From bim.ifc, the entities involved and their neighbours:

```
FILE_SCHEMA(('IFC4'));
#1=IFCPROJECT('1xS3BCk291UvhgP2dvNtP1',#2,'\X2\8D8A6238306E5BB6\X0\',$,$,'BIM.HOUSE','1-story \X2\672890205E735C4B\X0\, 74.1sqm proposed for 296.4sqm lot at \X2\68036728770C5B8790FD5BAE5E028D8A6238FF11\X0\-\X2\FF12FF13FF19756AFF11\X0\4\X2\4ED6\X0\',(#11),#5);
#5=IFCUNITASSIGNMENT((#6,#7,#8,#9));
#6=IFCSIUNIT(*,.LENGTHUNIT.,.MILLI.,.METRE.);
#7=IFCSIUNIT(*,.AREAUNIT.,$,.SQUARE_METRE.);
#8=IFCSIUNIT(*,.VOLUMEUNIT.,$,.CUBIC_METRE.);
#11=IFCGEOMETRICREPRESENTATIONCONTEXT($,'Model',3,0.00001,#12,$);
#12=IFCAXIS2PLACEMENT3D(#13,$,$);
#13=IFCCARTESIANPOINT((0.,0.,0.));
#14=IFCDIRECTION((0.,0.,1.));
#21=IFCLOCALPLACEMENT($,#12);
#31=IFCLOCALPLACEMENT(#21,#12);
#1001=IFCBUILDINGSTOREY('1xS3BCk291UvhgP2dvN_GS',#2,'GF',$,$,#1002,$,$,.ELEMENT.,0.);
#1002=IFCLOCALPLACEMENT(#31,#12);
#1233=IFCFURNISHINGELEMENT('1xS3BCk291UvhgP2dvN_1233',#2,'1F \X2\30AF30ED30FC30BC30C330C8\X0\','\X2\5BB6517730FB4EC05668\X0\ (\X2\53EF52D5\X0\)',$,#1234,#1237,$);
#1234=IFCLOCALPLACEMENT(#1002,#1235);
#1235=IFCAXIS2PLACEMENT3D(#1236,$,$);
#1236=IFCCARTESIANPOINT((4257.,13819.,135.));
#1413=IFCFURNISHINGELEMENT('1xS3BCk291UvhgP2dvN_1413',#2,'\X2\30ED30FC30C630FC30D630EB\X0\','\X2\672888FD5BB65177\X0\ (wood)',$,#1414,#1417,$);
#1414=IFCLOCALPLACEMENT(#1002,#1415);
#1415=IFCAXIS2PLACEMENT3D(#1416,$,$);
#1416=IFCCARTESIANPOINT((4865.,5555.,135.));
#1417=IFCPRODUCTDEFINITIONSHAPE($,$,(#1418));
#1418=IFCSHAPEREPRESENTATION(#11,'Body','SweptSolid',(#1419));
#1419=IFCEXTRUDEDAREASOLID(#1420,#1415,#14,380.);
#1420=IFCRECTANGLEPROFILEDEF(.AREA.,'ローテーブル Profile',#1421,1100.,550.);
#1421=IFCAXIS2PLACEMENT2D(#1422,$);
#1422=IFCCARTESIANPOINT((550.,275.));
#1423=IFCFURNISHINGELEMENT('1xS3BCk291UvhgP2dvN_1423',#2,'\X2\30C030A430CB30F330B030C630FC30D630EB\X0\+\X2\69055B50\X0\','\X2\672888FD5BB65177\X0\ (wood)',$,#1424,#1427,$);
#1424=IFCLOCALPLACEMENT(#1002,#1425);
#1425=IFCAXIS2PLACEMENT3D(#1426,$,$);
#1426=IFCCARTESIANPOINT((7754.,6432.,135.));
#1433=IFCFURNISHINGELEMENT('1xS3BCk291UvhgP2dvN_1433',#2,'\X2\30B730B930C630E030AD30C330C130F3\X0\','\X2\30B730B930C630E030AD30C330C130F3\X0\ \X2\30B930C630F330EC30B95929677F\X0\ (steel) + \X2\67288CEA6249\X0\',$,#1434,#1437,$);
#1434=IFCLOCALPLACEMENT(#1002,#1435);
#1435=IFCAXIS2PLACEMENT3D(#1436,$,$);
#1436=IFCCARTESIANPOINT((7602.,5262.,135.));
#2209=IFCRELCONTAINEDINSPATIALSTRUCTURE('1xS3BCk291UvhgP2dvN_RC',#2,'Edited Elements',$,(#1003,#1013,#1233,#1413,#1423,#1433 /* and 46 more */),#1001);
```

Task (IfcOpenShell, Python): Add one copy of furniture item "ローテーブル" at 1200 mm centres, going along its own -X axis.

```python
import ifcopenshell
import ifcopenshell.api.geometry
import ifcopenshell.api.root
import ifcopenshell.util.element
import ifcopenshell.util.placement

model = ifcopenshell.open("bim.ifc")


def reuse_history(source, copy):
    """copy_class also copies each property set's owner history, people and application; keep the originals."""
    for rel in copy.IsDefinedBy:
        if rel.is_a("IfcRelDefinesByProperties") and (history := rel.RelatingPropertyDefinition.OwnerHistory):
            rel.RelatingPropertyDefinition.OwnerHistory = source.OwnerHistory
            ifcopenshell.util.element.remove_deep2(model, history)


source = model.by_guid("1xS3BCk291UvhgP2dvN_1413")
base = ifcopenshell.util.placement.get_local_placement(source.ObjectPlacement)
step = -base[:3, 0] * 1200.0

for i in range(1, 2):
    copy = ifcopenshell.api.root.copy_class(model, product=source)
    copy.Representation = ifcopenshell.util.element.copy_deep(
        model, source.Representation, exclude=["IfcGeometricRepresentationContext", "IfcRepresentationMap"]
    )
    reuse_history(source, copy)
    matrix = base.copy()
    matrix[:3, 3] += i * step
    print("added at", matrix[:3, 3].round(3) + 0.0)
    ifcopenshell.api.geometry.edit_object_placement(model, product=copy, matrix=matrix, is_si=False)

model.write("bim_v2.ifc")
```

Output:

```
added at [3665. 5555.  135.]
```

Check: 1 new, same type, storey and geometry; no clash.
